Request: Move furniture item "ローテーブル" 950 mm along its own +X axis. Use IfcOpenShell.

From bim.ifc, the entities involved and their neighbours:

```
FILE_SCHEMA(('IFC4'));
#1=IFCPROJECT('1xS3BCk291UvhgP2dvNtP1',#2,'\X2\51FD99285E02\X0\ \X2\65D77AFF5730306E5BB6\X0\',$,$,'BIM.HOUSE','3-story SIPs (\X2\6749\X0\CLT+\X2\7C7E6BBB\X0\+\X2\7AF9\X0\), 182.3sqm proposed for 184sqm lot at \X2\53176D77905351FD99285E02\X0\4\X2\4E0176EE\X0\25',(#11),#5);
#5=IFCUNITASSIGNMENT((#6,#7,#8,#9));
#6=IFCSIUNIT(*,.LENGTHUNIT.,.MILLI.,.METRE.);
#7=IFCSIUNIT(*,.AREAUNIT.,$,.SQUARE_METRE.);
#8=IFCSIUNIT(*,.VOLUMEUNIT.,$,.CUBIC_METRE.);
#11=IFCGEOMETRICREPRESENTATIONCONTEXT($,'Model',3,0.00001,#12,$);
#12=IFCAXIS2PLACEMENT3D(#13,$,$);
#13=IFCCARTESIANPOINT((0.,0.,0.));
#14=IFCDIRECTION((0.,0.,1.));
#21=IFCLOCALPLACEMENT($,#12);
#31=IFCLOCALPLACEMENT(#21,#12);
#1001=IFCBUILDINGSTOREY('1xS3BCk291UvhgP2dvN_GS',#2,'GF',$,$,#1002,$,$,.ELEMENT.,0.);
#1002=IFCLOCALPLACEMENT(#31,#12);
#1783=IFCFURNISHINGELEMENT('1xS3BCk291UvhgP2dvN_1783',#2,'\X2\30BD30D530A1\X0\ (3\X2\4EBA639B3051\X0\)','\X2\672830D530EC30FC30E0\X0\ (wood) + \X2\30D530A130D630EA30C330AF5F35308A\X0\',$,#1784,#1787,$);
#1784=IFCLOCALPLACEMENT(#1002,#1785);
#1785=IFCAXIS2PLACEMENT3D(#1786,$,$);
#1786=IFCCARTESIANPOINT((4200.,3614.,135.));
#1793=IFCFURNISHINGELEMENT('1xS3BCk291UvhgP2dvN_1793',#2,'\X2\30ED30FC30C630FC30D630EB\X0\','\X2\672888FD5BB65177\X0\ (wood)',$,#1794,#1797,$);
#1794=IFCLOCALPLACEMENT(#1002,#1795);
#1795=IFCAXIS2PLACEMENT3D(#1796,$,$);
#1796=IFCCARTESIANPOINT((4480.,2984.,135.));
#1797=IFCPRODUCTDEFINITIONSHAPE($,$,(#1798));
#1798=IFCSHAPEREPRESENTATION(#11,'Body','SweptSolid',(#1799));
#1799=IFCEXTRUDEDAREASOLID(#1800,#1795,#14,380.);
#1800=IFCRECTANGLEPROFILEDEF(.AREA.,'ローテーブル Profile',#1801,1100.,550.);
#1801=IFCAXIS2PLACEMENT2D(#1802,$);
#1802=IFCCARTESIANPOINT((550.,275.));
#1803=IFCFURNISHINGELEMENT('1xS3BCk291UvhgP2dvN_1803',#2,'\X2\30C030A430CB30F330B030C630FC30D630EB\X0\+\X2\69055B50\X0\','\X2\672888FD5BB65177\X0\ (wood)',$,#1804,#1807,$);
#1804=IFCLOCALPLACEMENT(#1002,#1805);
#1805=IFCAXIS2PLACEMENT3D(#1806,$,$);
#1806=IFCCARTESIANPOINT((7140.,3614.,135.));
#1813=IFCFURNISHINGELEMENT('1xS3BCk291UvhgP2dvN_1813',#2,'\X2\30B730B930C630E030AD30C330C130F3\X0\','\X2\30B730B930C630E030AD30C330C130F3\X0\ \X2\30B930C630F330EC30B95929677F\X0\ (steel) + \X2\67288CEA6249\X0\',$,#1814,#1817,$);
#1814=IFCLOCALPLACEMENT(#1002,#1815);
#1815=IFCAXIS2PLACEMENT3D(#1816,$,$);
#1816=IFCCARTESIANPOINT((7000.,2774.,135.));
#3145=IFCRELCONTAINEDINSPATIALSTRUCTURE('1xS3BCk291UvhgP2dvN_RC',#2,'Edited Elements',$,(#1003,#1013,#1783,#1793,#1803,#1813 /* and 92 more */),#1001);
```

```python
import ifcopenshell
import ifcopenshell.api.geometry
import ifcopenshell.util.placement

model = ifcopenshell.open("bim.ifc")

item = model.by_id(1793)
matrix = ifcopenshell.util.placement.get_local_placement(item.ObjectPlacement)
matrix[:3, 3] += matrix[:3, 0] * 950.0
ifcopenshell.api.geometry.edit_object_placement(model, product=item, matrix=matrix, is_si=False)

print(ifcopenshell.util.placement.get_local_placement(item.ObjectPlacement).round(3) + 0.0)

model.write("bim_edited.ifc")
```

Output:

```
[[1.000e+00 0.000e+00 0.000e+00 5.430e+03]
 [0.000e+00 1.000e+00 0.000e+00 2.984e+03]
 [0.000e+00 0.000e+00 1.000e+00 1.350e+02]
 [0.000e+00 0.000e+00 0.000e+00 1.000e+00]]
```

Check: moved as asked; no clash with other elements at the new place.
